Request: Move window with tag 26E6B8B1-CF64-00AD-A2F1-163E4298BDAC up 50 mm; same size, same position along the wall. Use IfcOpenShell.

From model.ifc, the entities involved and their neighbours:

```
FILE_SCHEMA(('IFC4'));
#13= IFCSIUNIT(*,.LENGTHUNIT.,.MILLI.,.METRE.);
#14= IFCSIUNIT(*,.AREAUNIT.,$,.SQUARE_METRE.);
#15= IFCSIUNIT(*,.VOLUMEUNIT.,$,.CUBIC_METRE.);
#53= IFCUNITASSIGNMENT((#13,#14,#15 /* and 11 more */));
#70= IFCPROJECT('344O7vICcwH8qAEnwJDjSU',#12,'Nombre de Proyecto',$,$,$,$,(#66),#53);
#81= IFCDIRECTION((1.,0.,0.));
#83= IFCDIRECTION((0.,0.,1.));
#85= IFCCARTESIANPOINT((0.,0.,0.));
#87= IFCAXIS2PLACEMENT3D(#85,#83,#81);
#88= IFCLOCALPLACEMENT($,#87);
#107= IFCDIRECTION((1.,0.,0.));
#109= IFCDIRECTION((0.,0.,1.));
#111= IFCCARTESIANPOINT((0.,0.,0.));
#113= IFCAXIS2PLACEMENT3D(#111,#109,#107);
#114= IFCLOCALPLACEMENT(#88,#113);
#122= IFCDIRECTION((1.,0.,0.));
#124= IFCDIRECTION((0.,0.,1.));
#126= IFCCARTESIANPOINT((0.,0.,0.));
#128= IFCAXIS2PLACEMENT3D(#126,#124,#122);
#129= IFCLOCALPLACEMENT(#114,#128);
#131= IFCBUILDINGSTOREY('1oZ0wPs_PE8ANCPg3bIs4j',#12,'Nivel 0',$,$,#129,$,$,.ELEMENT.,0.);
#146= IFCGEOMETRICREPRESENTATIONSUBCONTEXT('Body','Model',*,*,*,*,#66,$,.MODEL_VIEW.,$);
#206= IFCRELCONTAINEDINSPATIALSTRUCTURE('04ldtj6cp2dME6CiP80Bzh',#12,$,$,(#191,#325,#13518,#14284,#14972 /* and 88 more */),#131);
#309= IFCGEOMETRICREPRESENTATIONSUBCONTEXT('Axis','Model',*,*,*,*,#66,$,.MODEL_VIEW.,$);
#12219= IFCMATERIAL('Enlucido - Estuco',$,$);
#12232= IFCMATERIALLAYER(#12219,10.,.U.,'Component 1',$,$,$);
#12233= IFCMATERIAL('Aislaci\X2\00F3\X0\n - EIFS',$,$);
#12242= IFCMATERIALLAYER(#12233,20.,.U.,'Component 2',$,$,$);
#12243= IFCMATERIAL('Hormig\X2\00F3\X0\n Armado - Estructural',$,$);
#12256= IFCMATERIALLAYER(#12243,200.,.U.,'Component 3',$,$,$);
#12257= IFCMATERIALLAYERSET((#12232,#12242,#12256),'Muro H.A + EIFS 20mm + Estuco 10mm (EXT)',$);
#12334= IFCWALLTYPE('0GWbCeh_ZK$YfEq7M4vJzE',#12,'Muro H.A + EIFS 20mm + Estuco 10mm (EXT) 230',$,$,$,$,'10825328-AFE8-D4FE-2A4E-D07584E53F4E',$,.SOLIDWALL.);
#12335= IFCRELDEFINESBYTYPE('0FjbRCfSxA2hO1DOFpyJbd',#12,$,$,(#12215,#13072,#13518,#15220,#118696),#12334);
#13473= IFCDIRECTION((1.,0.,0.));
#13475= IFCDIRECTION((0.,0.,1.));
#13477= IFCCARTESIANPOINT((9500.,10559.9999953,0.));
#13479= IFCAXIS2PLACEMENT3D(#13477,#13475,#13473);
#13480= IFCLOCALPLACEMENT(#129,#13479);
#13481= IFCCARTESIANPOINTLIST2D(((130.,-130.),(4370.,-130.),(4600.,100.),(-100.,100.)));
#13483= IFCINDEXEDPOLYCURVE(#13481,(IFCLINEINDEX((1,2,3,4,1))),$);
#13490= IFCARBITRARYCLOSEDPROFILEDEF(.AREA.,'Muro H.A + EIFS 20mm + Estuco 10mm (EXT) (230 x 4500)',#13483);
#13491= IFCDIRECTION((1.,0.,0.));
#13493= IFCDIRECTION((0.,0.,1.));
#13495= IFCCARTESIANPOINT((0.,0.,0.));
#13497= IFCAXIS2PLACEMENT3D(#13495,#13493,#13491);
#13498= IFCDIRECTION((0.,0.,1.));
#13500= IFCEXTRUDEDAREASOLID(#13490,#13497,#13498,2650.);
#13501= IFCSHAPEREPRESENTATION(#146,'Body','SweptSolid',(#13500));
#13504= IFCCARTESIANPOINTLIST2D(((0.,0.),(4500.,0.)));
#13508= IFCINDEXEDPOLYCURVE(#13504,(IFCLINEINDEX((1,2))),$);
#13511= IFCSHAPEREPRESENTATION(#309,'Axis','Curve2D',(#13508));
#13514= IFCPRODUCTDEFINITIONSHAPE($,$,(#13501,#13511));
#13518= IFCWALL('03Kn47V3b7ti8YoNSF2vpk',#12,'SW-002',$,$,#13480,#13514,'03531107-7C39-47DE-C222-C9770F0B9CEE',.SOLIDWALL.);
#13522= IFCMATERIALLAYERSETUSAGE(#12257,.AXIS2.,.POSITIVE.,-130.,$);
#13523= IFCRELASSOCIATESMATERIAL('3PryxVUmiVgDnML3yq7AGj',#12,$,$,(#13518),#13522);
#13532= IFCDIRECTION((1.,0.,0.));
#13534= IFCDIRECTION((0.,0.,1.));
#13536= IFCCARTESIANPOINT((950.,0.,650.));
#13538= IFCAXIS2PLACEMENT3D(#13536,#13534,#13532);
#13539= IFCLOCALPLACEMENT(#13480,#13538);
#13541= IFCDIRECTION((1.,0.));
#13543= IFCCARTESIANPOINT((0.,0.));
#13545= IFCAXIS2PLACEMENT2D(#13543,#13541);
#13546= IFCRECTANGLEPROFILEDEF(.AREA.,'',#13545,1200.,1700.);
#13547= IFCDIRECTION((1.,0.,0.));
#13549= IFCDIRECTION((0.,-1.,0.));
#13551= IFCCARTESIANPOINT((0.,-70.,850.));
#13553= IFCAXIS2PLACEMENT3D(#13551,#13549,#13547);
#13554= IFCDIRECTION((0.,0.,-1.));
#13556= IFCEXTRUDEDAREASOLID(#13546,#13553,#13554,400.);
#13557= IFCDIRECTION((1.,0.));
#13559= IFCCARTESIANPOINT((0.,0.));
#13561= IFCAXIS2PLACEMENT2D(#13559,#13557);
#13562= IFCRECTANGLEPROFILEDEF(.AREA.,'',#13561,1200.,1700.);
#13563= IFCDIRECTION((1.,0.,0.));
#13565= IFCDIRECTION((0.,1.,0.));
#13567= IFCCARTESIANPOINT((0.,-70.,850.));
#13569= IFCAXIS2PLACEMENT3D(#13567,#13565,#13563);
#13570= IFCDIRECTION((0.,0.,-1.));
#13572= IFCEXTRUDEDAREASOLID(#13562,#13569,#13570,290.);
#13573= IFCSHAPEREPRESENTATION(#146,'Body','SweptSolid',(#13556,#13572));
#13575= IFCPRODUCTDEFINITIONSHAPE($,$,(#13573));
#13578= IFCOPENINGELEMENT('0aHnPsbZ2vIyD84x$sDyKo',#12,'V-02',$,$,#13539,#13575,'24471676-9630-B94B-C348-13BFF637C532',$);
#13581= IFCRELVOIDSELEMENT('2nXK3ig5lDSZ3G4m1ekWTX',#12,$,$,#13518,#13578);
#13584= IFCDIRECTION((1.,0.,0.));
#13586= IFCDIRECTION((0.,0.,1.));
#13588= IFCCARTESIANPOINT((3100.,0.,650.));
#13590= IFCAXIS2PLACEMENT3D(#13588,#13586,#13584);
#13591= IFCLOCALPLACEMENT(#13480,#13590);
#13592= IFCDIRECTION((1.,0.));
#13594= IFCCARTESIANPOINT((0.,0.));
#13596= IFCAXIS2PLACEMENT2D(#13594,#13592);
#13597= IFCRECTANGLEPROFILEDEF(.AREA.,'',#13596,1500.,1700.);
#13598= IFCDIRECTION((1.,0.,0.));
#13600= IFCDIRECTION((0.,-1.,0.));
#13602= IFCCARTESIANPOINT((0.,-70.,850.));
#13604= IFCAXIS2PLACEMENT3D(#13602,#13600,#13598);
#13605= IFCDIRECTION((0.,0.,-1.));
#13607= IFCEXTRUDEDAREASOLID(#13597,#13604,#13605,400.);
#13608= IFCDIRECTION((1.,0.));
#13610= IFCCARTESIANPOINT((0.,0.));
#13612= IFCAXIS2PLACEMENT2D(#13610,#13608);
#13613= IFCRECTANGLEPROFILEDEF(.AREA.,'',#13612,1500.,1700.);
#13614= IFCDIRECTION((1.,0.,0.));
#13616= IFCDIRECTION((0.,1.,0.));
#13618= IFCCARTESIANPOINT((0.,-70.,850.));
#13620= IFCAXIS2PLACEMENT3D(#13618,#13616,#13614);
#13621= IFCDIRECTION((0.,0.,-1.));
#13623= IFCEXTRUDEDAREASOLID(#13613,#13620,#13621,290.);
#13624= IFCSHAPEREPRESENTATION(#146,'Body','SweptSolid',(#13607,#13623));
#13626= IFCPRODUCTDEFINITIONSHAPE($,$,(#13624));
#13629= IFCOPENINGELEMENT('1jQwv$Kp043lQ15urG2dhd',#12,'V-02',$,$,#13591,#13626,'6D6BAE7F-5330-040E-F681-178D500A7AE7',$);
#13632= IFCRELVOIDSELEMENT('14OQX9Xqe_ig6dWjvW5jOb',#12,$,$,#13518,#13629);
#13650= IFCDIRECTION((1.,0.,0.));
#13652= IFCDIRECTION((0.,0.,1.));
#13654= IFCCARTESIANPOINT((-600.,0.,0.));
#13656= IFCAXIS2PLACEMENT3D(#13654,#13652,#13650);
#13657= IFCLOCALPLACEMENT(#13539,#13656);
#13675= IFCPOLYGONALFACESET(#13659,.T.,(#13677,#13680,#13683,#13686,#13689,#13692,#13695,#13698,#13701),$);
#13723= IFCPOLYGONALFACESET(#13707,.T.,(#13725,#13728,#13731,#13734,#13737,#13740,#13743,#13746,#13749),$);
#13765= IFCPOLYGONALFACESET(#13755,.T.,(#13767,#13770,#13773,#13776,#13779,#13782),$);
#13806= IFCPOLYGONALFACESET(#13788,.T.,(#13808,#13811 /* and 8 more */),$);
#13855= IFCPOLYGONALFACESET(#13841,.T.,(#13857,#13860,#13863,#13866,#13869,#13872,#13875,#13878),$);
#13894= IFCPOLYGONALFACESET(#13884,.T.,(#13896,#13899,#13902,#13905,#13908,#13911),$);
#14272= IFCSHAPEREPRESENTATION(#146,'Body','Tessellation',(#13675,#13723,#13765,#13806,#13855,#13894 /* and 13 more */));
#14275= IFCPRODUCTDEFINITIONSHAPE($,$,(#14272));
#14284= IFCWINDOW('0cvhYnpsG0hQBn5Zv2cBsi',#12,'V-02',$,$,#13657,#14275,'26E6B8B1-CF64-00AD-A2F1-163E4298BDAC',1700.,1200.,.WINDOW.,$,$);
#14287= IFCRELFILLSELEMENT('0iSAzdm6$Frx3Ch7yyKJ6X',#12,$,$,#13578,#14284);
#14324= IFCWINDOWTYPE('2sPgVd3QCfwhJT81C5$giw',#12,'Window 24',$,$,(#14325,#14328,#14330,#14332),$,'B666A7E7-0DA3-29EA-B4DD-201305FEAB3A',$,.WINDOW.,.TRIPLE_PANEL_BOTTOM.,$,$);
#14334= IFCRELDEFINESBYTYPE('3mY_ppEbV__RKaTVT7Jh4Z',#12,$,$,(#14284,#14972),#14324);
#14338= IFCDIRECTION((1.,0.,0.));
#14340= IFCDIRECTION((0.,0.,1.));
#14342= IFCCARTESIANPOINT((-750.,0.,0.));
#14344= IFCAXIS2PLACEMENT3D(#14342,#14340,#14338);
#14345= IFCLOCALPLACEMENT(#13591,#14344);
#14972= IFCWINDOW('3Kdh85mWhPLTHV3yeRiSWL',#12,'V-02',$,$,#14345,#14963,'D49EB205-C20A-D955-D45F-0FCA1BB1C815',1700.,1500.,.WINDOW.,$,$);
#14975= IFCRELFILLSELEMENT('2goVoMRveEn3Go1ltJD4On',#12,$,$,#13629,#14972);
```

```python
import numpy as np
import ifcopenshell
import ifcopenshell.api.geometry
import ifcopenshell.util.placement
import ifcopenshell.util.unit

model = ifcopenshell.open("model.ifc")
unit_scale = ifcopenshell.util.unit.calculate_unit_scale(model)

window = model.by_id(14284)
opening = window.FillsVoids[0].RelatingOpeningElement
dz = 0.05 / unit_scale

shift = np.array([0.0, 0.0, dz])
# The window is placed relative to its opening, so it follows when the opening moves.
matrix = ifcopenshell.util.placement.get_local_placement(opening.ObjectPlacement)
matrix[:3, 3] += shift
ifcopenshell.api.geometry.edit_object_placement(
    model, product=opening, matrix=matrix, is_si=False, should_transform_children=True
)

print(f"moved by {dz * unit_scale:+.3f} m")

model.write("model_rev.ifc")
```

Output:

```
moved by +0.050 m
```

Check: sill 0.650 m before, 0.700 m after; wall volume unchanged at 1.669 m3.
